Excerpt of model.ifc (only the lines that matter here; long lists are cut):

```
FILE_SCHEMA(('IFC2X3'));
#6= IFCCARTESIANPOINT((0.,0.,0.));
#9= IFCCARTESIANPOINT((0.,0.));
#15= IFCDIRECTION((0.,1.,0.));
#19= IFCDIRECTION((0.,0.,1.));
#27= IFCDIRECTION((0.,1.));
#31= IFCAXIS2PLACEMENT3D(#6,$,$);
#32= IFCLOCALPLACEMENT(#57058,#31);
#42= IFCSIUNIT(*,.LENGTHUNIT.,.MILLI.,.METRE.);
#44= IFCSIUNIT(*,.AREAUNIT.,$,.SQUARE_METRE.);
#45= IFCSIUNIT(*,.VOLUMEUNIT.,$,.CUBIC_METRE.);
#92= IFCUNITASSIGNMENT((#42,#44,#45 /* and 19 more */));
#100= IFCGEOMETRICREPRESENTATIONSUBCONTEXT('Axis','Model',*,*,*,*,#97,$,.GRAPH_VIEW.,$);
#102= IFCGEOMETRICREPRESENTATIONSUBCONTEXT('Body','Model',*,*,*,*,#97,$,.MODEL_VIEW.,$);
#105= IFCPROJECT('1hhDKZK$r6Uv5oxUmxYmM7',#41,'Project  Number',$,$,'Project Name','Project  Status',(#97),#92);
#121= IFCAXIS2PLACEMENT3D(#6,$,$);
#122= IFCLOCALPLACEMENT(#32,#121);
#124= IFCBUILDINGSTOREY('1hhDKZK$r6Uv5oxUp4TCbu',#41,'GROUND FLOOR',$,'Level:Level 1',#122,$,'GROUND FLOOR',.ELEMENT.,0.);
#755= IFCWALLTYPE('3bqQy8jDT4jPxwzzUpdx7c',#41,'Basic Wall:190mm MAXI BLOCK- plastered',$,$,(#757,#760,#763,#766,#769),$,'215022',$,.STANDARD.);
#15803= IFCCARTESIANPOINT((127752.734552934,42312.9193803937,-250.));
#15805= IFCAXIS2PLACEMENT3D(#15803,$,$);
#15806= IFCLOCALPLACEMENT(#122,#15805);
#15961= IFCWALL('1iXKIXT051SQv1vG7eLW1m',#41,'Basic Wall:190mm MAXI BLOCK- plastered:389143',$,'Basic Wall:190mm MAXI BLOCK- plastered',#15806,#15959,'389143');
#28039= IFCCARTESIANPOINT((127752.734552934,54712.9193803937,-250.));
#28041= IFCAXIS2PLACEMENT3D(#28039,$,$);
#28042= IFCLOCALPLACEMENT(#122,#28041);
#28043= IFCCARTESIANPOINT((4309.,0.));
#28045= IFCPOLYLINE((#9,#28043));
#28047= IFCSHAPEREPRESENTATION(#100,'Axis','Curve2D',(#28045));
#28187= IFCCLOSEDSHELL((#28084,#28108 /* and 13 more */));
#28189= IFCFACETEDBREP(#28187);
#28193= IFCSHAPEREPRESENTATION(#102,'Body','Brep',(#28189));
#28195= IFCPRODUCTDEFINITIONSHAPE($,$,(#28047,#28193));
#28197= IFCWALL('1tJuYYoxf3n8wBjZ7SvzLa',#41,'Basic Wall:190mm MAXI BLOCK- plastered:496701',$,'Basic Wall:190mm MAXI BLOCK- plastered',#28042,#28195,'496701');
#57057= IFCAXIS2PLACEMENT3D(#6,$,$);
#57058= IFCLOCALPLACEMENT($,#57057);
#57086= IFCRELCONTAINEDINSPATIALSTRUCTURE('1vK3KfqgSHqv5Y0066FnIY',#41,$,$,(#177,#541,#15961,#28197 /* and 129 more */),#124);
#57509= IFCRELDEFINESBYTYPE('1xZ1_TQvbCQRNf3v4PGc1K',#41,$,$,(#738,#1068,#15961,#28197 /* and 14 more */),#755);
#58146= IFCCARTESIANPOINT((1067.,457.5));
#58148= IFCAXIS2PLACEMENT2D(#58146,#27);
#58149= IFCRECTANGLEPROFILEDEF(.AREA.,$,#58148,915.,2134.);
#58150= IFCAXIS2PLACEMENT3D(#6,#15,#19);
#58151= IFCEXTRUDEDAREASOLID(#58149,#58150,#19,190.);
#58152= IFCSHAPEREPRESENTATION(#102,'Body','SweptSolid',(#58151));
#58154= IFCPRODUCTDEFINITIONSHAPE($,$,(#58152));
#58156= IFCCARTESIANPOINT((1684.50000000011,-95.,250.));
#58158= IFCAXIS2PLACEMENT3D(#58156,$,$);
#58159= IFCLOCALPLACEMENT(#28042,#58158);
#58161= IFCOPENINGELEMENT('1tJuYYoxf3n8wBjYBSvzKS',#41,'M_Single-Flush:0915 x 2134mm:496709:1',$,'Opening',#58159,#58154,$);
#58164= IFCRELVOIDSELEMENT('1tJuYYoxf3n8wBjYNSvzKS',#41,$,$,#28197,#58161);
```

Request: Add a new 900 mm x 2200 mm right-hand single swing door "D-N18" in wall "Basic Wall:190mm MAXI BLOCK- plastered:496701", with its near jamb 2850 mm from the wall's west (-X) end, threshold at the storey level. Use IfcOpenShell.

```python
import numpy as np
import ifcopenshell
import ifcopenshell.api.feature
import ifcopenshell.api.geometry
import ifcopenshell.api.root
import ifcopenshell.api.spatial
import ifcopenshell.api.type
import ifcopenshell.geom
import ifcopenshell.util.element
import ifcopenshell.util.placement
import ifcopenshell.util.representation
import ifcopenshell.util.shape
import ifcopenshell.util.unit

model = ifcopenshell.open("model.ifc")
unit_scale = ifcopenshell.util.unit.calculate_unit_scale(model)
settings = ifcopenshell.geom.settings()


def volume(element):
    """Net volume in cubic metres, openings subtracted."""
    shape = ifcopenshell.geom.create_shape(settings, element)
    return ifcopenshell.util.shape.get_volume(shape.geometry)


wall = model.by_id(28197)
storey = ifcopenshell.util.element.get_container(wall, ifc_class="IfcBuildingStorey")
context = ifcopenshell.util.representation.get_context(model, "Model", "Body", "MODEL_VIEW")
before = volume(wall)

width, height, from_end, sill = 0.9, 2.2, 2.85, 0.0  # metres

# The wall runs along its own X axis, and the end named is its -X end.
wall_shape = ifcopenshell.geom.create_shape(settings, wall)
x, y, z = ifcopenshell.util.shape.get_vertices(wall_shape.geometry).T
start = x.min() + from_end
face, thickness = float(y.min()), float(y.max() - y.min())
wall_matrix = ifcopenshell.util.placement.get_local_placement(wall.ObjectPlacement)
level = ifcopenshell.util.placement.get_local_placement(storey.ObjectPlacement)[2, 3]


def in_wall(x, y):
    """Placement at x, y metres in the wall's axes, at sill height."""
    matrix = wall_matrix.copy()
    matrix[:, 3] = wall_matrix @ np.array([x / unit_scale, y / unit_scale, 0.0, 1.0])
    matrix[2, 3] = level + sill / unit_scale
    return matrix


# Opening: a box that overshoots both wall faces by 50 mm.
opening = ifcopenshell.api.root.create_entity(model, ifc_class="IfcOpeningElement")
box = ifcopenshell.api.geometry.add_wall_representation(
    model, context=context, length=width, height=height, thickness=thickness + 0.1
)
ifcopenshell.api.geometry.assign_representation(model, product=opening, representation=box)
ifcopenshell.api.geometry.edit_object_placement(model, product=opening, matrix=in_wall(start, face - 0.05), is_si=False)
ifcopenshell.api.feature.add_feature(model, feature=opening, element=wall)

door = ifcopenshell.api.root.create_entity(model, ifc_class="IfcDoor", name="D-N18")
door.OverallWidth, door.OverallHeight = width / unit_scale, height / unit_scale
body = ifcopenshell.api.geometry.add_door_representation(
    model,
    context=context,
    overall_width=door.OverallWidth,
    overall_height=door.OverallHeight,
    operation_type="SINGLE_SWING_RIGHT",
    lining_properties={"LiningDepth": thickness / unit_scale, "ThresholdDepth": thickness / unit_scale},
)
ifcopenshell.api.geometry.assign_representation(model, product=door, representation=body)
ifcopenshell.api.spatial.assign_container(model, products=[door], relating_structure=storey)
fills = ifcopenshell.api.feature.add_filling(model, opening=opening, element=door)
fills.OwnerHistory = door.OwnerHistory  # required in IFC2X3

# IFC2X3 keeps the operation on the door style.
style = ifcopenshell.api.root.create_entity(model, ifc_class="IfcDoorStyle", name="D-N18")
style.OperationType, style.ConstructionType = "SINGLE_SWING_RIGHT", "NOTDEFINED"
style.ParameterTakesPrecedence = style.Sizeable = False
ifcopenshell.api.type.assign_type(model, related_objects=[door], relating_type=style)

# The lining spans the wall, so the door starts at the wall face.
ifcopenshell.api.geometry.edit_object_placement(model, product=door, matrix=in_wall(start, face), is_si=False)

after = volume(wall)

print(f"wall volume {before:.3f} -> {after:.3f} m3")

model.write("model_v2.ifc")
```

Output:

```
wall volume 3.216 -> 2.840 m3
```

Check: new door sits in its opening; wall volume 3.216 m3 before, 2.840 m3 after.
